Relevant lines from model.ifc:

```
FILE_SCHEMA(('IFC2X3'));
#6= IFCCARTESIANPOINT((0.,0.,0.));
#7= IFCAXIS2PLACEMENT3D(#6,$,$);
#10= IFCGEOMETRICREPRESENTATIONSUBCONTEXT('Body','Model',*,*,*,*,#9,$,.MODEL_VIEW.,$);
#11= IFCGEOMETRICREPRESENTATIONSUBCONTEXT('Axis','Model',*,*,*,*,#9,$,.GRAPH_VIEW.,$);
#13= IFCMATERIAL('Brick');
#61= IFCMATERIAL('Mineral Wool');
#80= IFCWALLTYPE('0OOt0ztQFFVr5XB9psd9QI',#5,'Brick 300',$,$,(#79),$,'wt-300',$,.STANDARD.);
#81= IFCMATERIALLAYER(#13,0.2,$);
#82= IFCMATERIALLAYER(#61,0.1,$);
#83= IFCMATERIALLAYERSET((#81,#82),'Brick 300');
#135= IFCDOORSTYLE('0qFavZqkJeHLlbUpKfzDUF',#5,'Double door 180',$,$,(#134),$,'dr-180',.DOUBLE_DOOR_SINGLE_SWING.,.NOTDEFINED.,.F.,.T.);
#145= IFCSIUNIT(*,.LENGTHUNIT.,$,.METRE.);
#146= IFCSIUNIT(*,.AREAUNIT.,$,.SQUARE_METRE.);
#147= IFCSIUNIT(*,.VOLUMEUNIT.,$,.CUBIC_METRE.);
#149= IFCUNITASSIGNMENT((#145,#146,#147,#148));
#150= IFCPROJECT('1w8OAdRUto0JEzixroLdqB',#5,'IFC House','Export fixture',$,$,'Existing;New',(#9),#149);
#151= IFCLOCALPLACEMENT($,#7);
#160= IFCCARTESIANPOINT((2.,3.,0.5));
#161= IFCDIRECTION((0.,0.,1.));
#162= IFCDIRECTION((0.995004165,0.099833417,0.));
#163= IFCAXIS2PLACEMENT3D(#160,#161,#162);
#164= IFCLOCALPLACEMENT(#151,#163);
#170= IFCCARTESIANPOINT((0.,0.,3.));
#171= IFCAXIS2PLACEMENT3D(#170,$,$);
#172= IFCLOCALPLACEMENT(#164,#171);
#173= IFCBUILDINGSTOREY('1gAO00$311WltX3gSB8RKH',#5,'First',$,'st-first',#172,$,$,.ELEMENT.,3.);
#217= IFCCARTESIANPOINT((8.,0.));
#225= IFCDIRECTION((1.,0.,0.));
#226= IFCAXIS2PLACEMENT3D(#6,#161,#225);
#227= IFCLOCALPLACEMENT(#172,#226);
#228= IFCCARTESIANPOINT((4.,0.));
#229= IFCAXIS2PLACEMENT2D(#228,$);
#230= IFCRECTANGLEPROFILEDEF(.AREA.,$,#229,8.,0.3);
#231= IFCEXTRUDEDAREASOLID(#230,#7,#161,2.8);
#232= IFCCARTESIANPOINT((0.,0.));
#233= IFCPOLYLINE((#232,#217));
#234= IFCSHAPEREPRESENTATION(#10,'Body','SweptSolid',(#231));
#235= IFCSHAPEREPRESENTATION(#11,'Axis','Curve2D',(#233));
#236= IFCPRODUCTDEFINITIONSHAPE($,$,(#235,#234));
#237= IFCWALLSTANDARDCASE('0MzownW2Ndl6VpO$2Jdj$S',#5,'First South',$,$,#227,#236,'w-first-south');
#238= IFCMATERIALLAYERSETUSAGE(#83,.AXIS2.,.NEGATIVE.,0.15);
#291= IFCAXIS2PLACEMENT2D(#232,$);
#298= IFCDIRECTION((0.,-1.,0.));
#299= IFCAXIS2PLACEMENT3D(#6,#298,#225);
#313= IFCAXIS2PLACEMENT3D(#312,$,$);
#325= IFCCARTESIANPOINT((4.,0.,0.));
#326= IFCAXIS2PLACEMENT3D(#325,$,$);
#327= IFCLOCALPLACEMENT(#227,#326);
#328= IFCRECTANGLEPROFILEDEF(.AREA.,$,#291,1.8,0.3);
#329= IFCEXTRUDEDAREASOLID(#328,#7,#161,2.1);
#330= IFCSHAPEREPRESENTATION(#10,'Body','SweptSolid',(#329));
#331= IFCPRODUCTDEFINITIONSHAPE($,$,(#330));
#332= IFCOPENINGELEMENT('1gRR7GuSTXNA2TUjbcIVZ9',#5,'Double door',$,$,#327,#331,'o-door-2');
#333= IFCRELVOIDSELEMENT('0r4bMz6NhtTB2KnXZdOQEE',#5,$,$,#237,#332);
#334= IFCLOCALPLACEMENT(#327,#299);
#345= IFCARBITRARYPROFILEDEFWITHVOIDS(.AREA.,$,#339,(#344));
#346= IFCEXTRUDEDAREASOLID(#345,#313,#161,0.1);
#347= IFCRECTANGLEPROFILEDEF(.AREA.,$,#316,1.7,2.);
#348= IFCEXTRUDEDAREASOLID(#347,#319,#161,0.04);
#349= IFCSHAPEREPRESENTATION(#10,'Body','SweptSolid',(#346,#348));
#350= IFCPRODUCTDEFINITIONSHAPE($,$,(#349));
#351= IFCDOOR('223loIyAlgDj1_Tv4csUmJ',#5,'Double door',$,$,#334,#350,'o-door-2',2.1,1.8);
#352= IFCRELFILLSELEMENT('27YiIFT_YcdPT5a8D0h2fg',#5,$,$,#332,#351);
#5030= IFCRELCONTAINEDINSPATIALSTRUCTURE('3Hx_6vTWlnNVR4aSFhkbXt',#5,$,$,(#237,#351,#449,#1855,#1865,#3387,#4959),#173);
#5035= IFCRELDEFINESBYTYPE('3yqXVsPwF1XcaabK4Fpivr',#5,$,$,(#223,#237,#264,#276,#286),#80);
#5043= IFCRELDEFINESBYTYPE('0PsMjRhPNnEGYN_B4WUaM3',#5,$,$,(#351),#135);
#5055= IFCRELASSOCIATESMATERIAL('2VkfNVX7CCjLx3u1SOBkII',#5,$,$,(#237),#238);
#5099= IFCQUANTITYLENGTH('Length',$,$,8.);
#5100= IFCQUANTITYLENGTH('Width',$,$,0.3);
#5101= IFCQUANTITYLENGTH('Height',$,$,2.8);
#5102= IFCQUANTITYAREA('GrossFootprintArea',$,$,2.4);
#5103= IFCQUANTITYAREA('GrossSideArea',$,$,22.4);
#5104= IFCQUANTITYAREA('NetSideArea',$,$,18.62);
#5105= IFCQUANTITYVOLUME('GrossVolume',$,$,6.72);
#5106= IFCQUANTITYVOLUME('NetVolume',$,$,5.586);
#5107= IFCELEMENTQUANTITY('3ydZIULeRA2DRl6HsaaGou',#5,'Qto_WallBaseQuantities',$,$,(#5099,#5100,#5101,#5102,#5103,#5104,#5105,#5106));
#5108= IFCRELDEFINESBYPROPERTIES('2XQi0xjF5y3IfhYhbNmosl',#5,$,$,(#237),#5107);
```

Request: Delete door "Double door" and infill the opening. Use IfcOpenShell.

```python
import ifcopenshell
import ifcopenshell.api.feature
import ifcopenshell.api.pset
import ifcopenshell.api.root
import ifcopenshell.geom
import ifcopenshell.util.element
import ifcopenshell.util.shape
import ifcopenshell.util.unit

model = ifcopenshell.open("model.ifc")
area_scale = ifcopenshell.util.unit.calculate_unit_scale(model, "AREAUNIT")
volume_scale = ifcopenshell.util.unit.calculate_unit_scale(model, "VOLUMEUNIT")
settings = ifcopenshell.geom.settings()


def volume(element):
    """Net volume in cubic metres, openings subtracted."""
    shape = ifcopenshell.geom.create_shape(settings, element)
    return ifcopenshell.util.shape.get_volume(shape.geometry)


door = model.by_guid("223loIyAlgDj1_Tv4csUmJ")
opening = door.FillsVoids[0].RelatingOpeningElement
wall = opening.VoidsElements[0].RelatingBuildingElement
before = volume(wall)

ifcopenshell.api.root.remove_product(model, product=door)
ifcopenshell.api.feature.remove_feature(model, feature=opening)

after = volume(wall)
thickness = 0.3  # wall thickness in metres

# Update the wall's stored quantities.
qto = model.by_id(ifcopenshell.util.element.get_pset(wall, "Qto_WallBaseQuantities", should_inherit=False)["id"])
ifcopenshell.api.pset.edit_qto(model, qto=qto, properties={
    "NetSideArea": after / thickness / area_scale,
    "NetVolume": after / volume_scale,
})

print(f"wall volume {before:.3f} -> {after:.3f} m3")

model.write("model_edited.ifc")
```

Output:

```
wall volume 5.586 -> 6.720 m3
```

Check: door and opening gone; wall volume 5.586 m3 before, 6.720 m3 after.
